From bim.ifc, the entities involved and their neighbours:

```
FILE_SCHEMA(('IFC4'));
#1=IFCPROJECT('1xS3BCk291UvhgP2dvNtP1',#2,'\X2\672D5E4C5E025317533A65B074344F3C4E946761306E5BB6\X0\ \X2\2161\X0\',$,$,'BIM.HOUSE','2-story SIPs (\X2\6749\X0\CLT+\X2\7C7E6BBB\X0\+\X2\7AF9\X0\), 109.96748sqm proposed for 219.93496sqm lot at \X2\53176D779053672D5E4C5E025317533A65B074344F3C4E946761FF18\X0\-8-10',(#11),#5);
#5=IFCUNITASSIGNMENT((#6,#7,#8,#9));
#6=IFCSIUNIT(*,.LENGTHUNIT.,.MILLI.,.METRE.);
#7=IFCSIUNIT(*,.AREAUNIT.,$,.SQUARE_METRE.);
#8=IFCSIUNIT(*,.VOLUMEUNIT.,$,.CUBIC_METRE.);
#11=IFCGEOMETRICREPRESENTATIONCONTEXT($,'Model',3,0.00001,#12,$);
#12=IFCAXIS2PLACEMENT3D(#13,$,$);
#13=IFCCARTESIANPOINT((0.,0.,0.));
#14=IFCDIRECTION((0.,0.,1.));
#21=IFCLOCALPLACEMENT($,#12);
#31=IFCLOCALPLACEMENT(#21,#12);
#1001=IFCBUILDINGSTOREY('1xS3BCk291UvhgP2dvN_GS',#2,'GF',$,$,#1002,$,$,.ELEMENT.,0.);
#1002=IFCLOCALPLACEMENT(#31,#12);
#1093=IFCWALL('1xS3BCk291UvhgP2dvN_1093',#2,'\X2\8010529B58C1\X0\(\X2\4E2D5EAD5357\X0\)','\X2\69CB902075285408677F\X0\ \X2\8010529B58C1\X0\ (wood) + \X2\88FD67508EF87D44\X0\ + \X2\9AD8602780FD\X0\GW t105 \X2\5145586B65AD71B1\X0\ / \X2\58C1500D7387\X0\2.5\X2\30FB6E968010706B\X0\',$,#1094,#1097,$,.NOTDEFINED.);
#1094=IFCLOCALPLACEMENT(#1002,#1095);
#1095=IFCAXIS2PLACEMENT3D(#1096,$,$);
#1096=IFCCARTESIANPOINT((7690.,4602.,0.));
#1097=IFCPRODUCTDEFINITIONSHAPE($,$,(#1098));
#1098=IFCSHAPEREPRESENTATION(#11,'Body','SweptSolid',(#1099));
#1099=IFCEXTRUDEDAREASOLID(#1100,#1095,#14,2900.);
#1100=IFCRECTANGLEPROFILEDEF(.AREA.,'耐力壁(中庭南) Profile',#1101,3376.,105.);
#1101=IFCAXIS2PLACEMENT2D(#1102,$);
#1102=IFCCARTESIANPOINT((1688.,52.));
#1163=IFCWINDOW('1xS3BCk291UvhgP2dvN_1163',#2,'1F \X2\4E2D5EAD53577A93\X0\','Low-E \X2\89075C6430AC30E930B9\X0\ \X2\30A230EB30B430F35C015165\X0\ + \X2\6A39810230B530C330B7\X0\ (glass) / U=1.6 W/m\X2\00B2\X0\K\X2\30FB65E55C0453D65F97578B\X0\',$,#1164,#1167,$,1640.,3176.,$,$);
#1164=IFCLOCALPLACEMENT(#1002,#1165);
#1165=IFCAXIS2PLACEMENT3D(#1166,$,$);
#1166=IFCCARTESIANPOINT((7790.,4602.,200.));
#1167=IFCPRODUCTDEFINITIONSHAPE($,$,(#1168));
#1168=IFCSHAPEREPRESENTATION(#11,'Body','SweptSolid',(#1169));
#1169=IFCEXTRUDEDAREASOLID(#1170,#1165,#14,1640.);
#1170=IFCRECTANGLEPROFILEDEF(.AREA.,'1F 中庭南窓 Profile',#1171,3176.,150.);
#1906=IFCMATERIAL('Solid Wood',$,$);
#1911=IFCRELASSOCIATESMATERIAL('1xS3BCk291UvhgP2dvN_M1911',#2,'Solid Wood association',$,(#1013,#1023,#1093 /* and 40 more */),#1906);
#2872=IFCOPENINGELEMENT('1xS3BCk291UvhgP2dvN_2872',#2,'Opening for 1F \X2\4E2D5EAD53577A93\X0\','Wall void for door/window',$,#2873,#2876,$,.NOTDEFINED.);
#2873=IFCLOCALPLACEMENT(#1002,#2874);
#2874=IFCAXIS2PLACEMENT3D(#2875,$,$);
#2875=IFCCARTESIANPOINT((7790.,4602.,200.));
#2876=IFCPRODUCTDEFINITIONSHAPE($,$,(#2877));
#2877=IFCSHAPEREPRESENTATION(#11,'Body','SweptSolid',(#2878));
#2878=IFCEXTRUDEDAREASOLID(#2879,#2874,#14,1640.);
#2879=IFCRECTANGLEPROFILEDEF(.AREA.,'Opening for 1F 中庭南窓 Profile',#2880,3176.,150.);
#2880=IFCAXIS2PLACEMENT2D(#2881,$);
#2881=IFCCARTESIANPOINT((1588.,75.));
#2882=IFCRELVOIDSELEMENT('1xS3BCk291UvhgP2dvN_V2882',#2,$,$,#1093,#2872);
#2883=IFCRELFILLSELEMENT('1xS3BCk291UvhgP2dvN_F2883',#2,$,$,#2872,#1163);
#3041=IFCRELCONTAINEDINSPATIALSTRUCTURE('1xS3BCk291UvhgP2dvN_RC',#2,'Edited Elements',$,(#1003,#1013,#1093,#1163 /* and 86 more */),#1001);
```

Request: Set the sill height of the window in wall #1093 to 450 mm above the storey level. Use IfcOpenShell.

```python
import numpy as np
import ifcopenshell
import ifcopenshell.api.geometry
import ifcopenshell.geom
import ifcopenshell.util.element
import ifcopenshell.util.placement
import ifcopenshell.util.shape
import ifcopenshell.util.unit

model = ifcopenshell.open("bim.ifc")
unit_scale = ifcopenshell.util.unit.calculate_unit_scale(model)

window = model.by_guid("1xS3BCk291UvhgP2dvN_1163")
opening = window.FillsVoids[0].RelatingOpeningElement
storey = ifcopenshell.util.element.get_container(window, ifc_class="IfcBuildingStorey")
level = ifcopenshell.util.placement.get_local_placement(storey.ObjectPlacement)[2, 3]

# The opening's origin need not be at the sill, so measure its lowest point.
shape = ifcopenshell.geom.create_shape(ifcopenshell.geom.settings(), opening)
bottom = ifcopenshell.util.shape.get_shape_bottom_elevation(shape, shape.geometry) / unit_scale
dz = level + 0.45 / unit_scale - bottom

shift = np.array([0.0, 0.0, dz])
# The window is not placed relative to its opening, so move both.
for product in (opening, window):
    matrix = ifcopenshell.util.placement.get_local_placement(product.ObjectPlacement)
    matrix[:3, 3] += shift
    ifcopenshell.api.geometry.edit_object_placement(model, product=product, matrix=matrix, is_si=False)

print(f"moved by {dz * unit_scale:+.3f} m")

model.write("bim_edited.ifc")
```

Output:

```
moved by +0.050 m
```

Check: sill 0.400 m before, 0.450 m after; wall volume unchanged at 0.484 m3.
